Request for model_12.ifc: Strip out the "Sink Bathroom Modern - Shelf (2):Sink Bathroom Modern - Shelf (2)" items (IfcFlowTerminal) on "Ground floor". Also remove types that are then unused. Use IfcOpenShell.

First a look at what the model holds.

```python
import ifcopenshell
import ifcopenshell.util.element

model = ifcopenshell.open("model_12.ifc")
print(model.schema)
storey = next(s for s in model.by_type("IfcBuildingStorey") if s.Name == "Ground floor")
terminals = [e for e in ifcopenshell.util.element.get_decomposition(storey) if e.is_a("IfcFlowTerminal")]
seen = {}
for e in terminals:
    element_type = ifcopenshell.util.element.get_type(e)
    name = element_type.Name if element_type not in (None, e) else None
    seen[name] = seen.get(name, 0) + 1
for name, count in sorted(seen.items(), key=str):
    print(count, "x", name)
```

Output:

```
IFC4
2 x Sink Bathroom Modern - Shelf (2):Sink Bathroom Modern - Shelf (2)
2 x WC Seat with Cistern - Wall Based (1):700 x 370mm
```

```python
import ifcopenshell
import ifcopenshell.api.root
import ifcopenshell.util.element

model = ifcopenshell.open("model_12.ifc")

storey = next(s for s in model.by_type("IfcBuildingStorey") if s.Name == "Ground floor")
terminals = [e for e in ifcopenshell.util.element.get_decomposition(storey) if e.is_a("IfcFlowTerminal")]
targets = [e for e in terminals if (t := ifcopenshell.util.element.get_type(e)) not in (None, e) and t.Name == "Sink Bathroom Modern - Shelf (2):Sink Bathroom Modern - Shelf (2)"]
types = {ifcopenshell.util.element.get_type(e) for e in targets} - {None, *targets}

for e in targets:
    ifcopenshell.api.root.remove_product(model, product=e)
print(len(targets), "removed")

unused = [t for t in types if not ifcopenshell.util.element.get_types(t)]
for t in unused:
    ifcopenshell.api.root.remove_product(model, product=t)
print(len(unused), "unused types removed")

model.write("model_12_updated.ifc")
```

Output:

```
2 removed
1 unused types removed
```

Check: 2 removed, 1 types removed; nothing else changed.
